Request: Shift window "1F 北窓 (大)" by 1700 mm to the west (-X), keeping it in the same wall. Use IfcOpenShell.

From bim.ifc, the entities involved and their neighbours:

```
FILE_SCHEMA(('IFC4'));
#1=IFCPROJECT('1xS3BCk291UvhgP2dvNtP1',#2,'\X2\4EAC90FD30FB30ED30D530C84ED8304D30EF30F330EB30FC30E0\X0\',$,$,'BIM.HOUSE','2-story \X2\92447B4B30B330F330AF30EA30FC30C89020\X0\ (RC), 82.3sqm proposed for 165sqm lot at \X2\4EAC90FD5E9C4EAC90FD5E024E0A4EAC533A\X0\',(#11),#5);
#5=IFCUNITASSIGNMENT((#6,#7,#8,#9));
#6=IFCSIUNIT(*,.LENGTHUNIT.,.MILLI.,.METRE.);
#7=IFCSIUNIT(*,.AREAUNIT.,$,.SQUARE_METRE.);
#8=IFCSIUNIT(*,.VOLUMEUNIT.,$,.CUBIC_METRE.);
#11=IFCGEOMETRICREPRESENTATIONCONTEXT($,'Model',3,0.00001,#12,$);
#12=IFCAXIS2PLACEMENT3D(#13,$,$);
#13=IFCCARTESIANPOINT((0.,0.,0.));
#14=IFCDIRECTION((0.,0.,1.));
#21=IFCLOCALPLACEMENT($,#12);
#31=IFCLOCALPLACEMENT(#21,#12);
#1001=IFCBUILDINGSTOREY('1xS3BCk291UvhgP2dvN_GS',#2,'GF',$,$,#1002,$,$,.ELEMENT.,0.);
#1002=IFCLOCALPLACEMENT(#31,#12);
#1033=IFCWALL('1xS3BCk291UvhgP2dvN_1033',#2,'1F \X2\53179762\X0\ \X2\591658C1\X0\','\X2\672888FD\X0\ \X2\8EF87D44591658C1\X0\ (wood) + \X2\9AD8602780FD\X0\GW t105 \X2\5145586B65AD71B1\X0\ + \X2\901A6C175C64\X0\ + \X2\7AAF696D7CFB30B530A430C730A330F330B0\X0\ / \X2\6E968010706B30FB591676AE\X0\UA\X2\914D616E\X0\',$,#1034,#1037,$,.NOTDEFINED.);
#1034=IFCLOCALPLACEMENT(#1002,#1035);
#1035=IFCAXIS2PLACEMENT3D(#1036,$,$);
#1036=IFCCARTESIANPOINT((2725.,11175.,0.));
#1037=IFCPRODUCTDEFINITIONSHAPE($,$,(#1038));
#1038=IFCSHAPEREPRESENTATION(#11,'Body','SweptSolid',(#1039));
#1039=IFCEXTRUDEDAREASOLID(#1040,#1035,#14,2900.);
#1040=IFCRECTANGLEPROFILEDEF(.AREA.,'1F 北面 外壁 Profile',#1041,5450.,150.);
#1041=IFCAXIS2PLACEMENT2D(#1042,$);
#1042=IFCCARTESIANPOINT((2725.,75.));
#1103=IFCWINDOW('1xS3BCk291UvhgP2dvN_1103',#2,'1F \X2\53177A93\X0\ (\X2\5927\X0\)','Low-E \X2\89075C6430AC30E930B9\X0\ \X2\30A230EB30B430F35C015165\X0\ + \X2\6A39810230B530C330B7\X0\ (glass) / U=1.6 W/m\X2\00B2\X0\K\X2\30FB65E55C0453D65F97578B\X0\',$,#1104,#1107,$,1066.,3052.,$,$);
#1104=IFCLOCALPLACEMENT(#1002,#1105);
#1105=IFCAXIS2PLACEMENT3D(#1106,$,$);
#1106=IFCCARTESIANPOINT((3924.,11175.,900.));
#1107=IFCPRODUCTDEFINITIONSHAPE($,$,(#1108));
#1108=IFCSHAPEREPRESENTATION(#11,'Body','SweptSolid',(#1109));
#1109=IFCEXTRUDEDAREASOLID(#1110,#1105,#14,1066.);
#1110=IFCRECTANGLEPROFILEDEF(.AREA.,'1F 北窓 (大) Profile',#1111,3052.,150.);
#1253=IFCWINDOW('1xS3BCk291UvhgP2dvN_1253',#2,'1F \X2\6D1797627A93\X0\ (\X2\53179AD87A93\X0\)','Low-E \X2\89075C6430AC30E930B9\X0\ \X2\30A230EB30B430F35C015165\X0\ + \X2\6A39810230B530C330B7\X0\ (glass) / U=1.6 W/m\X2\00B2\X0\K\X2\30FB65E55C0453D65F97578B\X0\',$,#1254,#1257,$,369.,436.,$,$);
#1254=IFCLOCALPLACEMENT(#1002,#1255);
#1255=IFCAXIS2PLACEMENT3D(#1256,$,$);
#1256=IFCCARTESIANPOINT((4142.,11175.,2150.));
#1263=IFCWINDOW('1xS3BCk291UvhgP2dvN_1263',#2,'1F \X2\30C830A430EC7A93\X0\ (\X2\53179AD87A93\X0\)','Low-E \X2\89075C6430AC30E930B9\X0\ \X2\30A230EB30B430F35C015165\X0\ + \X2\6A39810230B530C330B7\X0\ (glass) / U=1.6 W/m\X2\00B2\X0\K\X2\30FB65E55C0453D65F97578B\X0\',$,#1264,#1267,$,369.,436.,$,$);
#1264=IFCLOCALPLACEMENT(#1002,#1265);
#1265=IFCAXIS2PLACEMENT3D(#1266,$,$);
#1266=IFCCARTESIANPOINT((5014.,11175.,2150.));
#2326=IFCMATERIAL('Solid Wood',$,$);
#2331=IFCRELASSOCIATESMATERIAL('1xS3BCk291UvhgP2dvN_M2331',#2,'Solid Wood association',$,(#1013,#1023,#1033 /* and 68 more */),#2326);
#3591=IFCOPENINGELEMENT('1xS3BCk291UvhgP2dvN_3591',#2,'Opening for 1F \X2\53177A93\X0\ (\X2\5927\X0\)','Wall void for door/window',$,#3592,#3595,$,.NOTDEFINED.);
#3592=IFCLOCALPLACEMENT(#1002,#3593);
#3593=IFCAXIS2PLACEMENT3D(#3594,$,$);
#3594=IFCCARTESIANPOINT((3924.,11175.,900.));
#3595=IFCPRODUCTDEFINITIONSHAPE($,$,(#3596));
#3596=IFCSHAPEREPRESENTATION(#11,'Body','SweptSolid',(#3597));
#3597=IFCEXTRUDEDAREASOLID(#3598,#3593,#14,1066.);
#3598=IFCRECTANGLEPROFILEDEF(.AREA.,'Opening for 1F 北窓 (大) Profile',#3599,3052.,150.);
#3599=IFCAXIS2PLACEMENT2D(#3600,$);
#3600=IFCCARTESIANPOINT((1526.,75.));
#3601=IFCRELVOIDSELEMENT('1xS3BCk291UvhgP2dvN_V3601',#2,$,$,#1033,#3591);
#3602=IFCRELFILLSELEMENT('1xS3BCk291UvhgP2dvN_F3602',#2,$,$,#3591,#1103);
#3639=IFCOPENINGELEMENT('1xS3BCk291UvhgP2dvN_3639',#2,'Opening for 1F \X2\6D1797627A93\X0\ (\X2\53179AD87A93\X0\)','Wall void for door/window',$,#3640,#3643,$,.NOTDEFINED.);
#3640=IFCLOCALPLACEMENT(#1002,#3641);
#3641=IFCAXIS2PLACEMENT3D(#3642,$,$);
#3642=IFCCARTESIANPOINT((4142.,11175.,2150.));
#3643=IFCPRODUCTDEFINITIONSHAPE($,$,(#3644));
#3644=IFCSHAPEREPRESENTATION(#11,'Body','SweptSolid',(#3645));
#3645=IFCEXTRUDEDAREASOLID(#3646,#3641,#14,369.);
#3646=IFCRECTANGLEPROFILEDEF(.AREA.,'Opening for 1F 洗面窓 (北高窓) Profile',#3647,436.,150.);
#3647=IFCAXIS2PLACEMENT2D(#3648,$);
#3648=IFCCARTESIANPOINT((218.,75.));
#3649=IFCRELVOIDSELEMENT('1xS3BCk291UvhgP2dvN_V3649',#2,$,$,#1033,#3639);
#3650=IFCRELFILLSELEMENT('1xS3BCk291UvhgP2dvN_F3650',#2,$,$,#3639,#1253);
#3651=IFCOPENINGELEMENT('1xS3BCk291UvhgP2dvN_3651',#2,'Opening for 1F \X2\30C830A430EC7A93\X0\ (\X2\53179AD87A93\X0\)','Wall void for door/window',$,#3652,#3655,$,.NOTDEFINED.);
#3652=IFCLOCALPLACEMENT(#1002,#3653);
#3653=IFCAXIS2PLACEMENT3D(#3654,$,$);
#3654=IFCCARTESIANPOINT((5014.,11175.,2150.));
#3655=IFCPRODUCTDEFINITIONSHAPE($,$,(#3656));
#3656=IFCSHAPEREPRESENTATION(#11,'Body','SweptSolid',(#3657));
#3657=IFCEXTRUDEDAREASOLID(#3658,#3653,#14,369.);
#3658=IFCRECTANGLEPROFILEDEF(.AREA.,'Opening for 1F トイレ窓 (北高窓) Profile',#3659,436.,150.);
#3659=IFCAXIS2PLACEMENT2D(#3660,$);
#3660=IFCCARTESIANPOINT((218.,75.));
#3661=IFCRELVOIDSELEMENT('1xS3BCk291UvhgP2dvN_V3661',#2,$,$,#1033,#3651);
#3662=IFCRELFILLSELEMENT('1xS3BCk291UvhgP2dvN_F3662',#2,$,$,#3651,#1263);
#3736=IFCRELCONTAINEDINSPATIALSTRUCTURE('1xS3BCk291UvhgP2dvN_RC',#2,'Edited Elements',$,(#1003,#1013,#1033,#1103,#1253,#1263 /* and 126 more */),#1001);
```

```python
import ifcopenshell
import ifcopenshell.api.geometry
import ifcopenshell.util.placement
import ifcopenshell.util.unit

model = ifcopenshell.open("bim.ifc")
unit_scale = ifcopenshell.util.unit.calculate_unit_scale(model)

window = model.by_id(1103)
opening = window.FillsVoids[0].RelatingOpeningElement
wall = opening.VoidsElements[0].RelatingBuildingElement

wall_matrix = ifcopenshell.util.placement.get_local_placement(wall.ObjectPlacement)
shift = wall_matrix[:3, 0] * -1.7 / unit_scale
before = ifcopenshell.util.placement.get_local_placement(window.ObjectPlacement)[:3, 3].copy()

# The window is not placed relative to its opening, so move both.
for product in (opening, window):
    matrix = ifcopenshell.util.placement.get_local_placement(product.ObjectPlacement)
    matrix[:3, 3] += shift
    ifcopenshell.api.geometry.edit_object_placement(model, product=product, matrix=matrix, is_si=False)

after = ifcopenshell.util.placement.get_local_placement(window.ObjectPlacement)[:3, 3]
print("window moved by", (after - before).round(3) + 0.0)

model.write("bim_updated.ifc")
```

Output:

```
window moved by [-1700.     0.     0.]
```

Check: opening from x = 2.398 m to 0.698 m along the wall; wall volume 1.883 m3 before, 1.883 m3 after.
